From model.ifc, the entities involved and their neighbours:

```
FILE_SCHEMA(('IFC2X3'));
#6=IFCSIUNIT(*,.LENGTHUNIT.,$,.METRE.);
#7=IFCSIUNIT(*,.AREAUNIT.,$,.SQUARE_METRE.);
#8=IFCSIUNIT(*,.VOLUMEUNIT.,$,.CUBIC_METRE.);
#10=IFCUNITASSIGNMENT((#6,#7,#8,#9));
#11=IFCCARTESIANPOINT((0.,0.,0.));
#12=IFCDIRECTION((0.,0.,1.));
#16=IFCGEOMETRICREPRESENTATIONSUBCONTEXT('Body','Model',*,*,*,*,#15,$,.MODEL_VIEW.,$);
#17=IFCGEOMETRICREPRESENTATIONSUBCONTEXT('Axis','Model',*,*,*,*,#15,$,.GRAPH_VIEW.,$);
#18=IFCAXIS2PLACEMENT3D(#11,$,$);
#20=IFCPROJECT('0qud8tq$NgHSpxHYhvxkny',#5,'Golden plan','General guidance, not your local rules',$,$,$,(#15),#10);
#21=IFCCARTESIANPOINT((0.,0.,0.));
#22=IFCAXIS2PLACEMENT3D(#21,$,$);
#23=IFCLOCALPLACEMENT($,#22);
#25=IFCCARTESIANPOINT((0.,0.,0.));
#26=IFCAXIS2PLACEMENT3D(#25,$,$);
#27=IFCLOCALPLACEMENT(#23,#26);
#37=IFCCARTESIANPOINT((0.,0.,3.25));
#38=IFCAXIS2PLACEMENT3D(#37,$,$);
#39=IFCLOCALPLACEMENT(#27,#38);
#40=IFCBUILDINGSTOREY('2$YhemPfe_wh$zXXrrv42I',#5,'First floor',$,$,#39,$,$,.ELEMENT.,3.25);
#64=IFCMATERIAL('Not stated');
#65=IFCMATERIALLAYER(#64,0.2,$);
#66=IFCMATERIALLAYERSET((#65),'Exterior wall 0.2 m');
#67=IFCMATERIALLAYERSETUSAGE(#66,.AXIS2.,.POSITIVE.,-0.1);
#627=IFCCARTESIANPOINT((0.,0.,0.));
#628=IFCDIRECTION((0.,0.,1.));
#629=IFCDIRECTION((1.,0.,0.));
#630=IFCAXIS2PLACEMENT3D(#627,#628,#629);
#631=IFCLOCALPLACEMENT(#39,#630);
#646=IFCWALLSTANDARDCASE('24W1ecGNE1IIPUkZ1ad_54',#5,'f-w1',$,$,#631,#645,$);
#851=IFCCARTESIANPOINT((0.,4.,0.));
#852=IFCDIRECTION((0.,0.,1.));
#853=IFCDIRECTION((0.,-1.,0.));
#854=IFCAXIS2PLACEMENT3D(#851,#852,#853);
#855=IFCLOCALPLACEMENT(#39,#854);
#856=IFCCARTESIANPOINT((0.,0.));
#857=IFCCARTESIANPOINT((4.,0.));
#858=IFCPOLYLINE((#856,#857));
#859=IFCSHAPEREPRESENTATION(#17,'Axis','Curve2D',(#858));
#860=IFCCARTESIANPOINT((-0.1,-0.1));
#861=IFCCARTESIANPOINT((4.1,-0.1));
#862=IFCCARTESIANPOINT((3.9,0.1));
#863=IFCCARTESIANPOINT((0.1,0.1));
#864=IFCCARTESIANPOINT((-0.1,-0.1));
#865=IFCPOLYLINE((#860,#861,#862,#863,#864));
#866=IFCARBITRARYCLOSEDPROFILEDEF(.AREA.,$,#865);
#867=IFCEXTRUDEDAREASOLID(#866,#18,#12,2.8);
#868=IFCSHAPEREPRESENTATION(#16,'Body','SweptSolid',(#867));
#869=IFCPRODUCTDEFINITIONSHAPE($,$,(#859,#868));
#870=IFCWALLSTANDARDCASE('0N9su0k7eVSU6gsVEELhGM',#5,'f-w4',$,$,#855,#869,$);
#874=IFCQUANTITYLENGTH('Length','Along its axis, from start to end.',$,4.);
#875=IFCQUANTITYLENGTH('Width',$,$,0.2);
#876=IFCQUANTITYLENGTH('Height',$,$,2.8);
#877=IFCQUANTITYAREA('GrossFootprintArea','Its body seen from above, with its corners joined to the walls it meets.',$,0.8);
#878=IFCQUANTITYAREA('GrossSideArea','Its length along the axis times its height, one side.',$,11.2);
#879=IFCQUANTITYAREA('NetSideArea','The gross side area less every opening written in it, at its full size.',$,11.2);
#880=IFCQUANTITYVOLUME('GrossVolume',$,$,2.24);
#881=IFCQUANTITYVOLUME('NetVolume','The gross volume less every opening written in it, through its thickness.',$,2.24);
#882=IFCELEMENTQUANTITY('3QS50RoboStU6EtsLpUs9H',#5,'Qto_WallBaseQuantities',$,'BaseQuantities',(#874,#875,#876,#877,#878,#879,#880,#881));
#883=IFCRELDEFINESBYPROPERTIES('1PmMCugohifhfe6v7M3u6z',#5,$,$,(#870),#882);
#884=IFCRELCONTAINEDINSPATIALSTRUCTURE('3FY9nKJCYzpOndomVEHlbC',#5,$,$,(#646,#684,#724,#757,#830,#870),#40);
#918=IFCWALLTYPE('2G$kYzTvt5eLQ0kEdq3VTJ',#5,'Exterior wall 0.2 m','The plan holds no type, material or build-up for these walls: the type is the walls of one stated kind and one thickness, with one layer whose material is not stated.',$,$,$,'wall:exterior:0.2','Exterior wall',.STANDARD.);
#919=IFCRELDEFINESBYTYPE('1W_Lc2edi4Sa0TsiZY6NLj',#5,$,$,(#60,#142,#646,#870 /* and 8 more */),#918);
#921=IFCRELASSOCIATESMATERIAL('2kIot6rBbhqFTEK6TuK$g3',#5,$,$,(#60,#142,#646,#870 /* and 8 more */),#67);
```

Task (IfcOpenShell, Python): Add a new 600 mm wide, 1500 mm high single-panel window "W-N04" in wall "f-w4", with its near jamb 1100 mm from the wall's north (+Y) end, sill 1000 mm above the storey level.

```python
import numpy as np
import ifcopenshell
import ifcopenshell.api.feature
import ifcopenshell.api.geometry
import ifcopenshell.api.pset
import ifcopenshell.api.root
import ifcopenshell.api.spatial
import ifcopenshell.api.type
import ifcopenshell.geom
import ifcopenshell.util.element
import ifcopenshell.util.placement
import ifcopenshell.util.representation
import ifcopenshell.util.shape
import ifcopenshell.util.unit

model = ifcopenshell.open("model.ifc")
unit_scale = ifcopenshell.util.unit.calculate_unit_scale(model)
area_scale = ifcopenshell.util.unit.calculate_unit_scale(model, "AREAUNIT")
volume_scale = ifcopenshell.util.unit.calculate_unit_scale(model, "VOLUMEUNIT")
settings = ifcopenshell.geom.settings()


def volume(element):
    """Net volume in cubic metres, openings subtracted."""
    shape = ifcopenshell.geom.create_shape(settings, element)
    return ifcopenshell.util.shape.get_volume(shape.geometry)


wall = model.by_guid("0N9su0k7eVSU6gsVEELhGM")
storey = ifcopenshell.util.element.get_container(wall, ifc_class="IfcBuildingStorey")
context = ifcopenshell.util.representation.get_context(model, "Model", "Body", "MODEL_VIEW")
before = volume(wall)

width, height, from_end, sill = 0.6, 1.5, 1.1, 1  # metres

# The wall runs along its own X axis, and the end named is its -X end.
wall_shape = ifcopenshell.geom.create_shape(settings, wall)
x, y, z = ifcopenshell.util.shape.get_vertices(wall_shape.geometry).T
start = x.min() + from_end
face, thickness = float(y.min()), float(y.max() - y.min())
wall_matrix = ifcopenshell.util.placement.get_local_placement(wall.ObjectPlacement)
level = ifcopenshell.util.placement.get_local_placement(storey.ObjectPlacement)[2, 3]


def in_wall(x, y):
    """Placement at x, y metres in the wall's axes, at sill height."""
    matrix = wall_matrix.copy()
    matrix[:, 3] = wall_matrix @ np.array([x / unit_scale, y / unit_scale, 0.0, 1.0])
    matrix[2, 3] = level + sill / unit_scale
    return matrix


# Opening: a box that overshoots both wall faces by 50 mm.
opening = ifcopenshell.api.root.create_entity(model, ifc_class="IfcOpeningElement")
box = ifcopenshell.api.geometry.add_wall_representation(
    model, context=context, length=width, height=height, thickness=thickness + 0.1
)
ifcopenshell.api.geometry.assign_representation(model, product=opening, representation=box)
ifcopenshell.api.geometry.edit_object_placement(model, product=opening, matrix=in_wall(start, face - 0.05), is_si=False)
ifcopenshell.api.feature.add_feature(model, feature=opening, element=wall)

window = ifcopenshell.api.root.create_entity(model, ifc_class="IfcWindow", name="W-N04")
window.OverallWidth, window.OverallHeight = width / unit_scale, height / unit_scale
body = ifcopenshell.api.geometry.add_window_representation(
    model,
    context=context,
    overall_width=window.OverallWidth,
    overall_height=window.OverallHeight,
    partition_type="SINGLE_PANEL",
)
ifcopenshell.api.geometry.assign_representation(model, product=window, representation=body)
ifcopenshell.api.spatial.assign_container(model, products=[window], relating_structure=storey)
fills = ifcopenshell.api.feature.add_filling(model, opening=opening, element=window)
fills.OwnerHistory = window.OwnerHistory  # required in IFC2X3

# IFC2X3 keeps the operation on the window style.
style = ifcopenshell.api.root.create_entity(model, ifc_class="IfcWindowStyle", name="W-N04")
style.OperationType, style.ConstructionType = "SINGLE_PANEL", "NOTDEFINED"
style.ParameterTakesPrecedence = style.Sizeable = False
ifcopenshell.api.type.assign_type(model, related_objects=[window], relating_type=style)

# Centre the window in the wall's thickness.
ifcopenshell.api.geometry.edit_object_placement(model, product=window, matrix=in_wall(start, face), is_si=False)
window_shape = ifcopenshell.geom.create_shape(settings, window)
depth = ifcopenshell.util.shape.get_vertices(window_shape.geometry)[:, 1]
offset = face + thickness / 2 - (depth.min() + depth.max()) / 2
ifcopenshell.api.geometry.edit_object_placement(model, product=window, matrix=in_wall(start, offset), is_si=False)

after = volume(wall)

# Update the wall's stored quantities.
qto = model.by_id(ifcopenshell.util.element.get_pset(wall, "Qto_WallBaseQuantities", should_inherit=False)["id"])
ifcopenshell.api.pset.edit_qto(model, qto=qto, properties={
    "NetSideArea": after / thickness / area_scale,
    "NetVolume": after / volume_scale,
})

print(f"wall volume {before:.3f} -> {after:.3f} m3")

model.write("model_edited.ifc")
```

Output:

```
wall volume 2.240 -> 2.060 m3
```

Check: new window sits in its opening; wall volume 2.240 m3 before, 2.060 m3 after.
